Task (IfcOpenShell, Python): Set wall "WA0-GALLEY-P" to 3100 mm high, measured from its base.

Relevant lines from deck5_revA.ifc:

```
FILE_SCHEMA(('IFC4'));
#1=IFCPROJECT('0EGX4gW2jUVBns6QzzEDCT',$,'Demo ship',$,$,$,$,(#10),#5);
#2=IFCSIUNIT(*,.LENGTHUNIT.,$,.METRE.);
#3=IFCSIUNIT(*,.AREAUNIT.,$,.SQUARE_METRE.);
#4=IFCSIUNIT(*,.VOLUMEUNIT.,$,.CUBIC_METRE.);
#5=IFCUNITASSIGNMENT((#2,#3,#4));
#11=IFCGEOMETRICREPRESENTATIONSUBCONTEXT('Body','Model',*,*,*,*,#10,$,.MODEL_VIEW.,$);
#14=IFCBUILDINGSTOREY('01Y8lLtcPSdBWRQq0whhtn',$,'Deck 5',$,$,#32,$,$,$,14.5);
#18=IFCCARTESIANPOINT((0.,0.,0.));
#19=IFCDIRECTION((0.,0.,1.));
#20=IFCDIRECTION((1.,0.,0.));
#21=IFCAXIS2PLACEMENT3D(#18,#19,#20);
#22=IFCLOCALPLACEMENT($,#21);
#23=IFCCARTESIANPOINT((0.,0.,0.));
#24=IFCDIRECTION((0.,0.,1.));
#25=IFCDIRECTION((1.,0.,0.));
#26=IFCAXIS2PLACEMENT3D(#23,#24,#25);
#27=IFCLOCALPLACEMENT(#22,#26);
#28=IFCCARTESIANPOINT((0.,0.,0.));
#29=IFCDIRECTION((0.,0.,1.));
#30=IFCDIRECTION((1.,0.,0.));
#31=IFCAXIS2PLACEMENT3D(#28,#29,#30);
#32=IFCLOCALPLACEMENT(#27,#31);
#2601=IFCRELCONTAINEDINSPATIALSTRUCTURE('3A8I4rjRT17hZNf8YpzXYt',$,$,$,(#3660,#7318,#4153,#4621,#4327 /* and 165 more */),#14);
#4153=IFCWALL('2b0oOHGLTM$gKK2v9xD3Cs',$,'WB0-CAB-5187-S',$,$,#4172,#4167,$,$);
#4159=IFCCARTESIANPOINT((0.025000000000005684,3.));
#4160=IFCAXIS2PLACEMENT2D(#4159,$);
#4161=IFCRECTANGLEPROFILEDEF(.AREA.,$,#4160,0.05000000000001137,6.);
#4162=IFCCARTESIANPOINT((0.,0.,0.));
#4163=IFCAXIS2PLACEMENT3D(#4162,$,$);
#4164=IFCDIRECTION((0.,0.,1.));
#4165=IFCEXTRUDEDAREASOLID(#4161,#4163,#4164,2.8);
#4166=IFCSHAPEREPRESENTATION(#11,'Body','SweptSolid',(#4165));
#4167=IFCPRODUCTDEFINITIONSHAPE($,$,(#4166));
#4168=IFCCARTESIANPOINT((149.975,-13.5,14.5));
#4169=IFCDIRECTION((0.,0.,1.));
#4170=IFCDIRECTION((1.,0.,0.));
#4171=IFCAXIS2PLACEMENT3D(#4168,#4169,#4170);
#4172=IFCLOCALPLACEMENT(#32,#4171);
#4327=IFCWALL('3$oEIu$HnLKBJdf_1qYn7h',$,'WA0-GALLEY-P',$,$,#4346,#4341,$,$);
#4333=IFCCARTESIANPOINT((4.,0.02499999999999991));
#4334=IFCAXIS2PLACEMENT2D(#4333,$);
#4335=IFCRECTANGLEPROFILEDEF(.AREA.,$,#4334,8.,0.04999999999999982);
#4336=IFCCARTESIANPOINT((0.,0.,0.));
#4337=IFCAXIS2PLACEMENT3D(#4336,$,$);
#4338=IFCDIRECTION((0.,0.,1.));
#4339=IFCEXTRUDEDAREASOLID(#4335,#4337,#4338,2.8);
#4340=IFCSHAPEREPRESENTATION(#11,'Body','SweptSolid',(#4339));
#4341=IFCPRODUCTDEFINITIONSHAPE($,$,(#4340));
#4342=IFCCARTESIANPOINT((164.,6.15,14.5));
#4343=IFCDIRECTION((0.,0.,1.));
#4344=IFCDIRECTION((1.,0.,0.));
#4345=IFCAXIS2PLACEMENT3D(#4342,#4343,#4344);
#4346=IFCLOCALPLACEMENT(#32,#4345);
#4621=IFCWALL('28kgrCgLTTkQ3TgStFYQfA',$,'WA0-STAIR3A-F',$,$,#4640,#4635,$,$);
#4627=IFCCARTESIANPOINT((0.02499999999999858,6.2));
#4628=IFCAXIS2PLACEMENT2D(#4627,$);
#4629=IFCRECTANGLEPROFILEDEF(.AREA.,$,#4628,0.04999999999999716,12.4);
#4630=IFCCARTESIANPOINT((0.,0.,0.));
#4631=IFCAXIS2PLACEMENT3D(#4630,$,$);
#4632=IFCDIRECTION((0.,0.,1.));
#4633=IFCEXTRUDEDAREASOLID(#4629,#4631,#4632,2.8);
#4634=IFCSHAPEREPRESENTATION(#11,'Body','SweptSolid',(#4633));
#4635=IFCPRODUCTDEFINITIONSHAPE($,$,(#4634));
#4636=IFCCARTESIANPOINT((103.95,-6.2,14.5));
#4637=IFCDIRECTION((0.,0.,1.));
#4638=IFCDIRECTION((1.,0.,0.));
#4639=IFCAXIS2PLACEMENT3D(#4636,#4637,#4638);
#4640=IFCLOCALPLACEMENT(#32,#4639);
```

```python
import ifcopenshell
import ifcopenshell.geom
import ifcopenshell.util.representation
import ifcopenshell.util.shape
import ifcopenshell.util.unit

model = ifcopenshell.open("deck5_revA.ifc")
unit_scale = ifcopenshell.util.unit.calculate_unit_scale(model)
settings = ifcopenshell.geom.settings()


def volume(element):
    """Net volume in cubic metres, openings subtracted."""
    shape = ifcopenshell.geom.create_shape(settings, element)
    return ifcopenshell.util.shape.get_volume(shape.geometry)


wall = model.by_guid("3$oEIu$HnLKBJdf_1qYn7h")
before = volume(wall)

body = ifcopenshell.util.representation.get_representation(wall, "Model", "Body")
solid = body.Items[0]
old_height = solid.Depth
solid.Depth = 3.1 / unit_scale
after = volume(wall)

print(f"height {old_height:g} -> {solid.Depth:g}, volume {before:.3f} -> {after:.3f} m3")

model.write("deck5_revA-out.ifc")
```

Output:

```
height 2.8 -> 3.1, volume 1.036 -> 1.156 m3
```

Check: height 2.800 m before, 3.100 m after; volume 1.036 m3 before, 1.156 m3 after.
